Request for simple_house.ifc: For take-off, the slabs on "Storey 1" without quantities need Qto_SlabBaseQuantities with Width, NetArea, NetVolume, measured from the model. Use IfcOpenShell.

First a look at what the model holds.

```python
import ifcopenshell
import ifcopenshell.util.element
import ifcopenshell.util.unit

model = ifcopenshell.open("simple_house.ifc")
print(model.schema)
for unit_type in ("LENGTHUNIT", "AREAUNIT", "VOLUMEUNIT"):
    print(unit_type, ifcopenshell.util.unit.calculate_unit_scale(model, unit_type))
storey = next(s for s in model.by_type("IfcBuildingStorey") if s.Name == "Storey 1")
slabs = [e for e in ifcopenshell.util.element.get_decomposition(storey) if e.is_a("IfcSlab")]
for e in sorted(slabs, key=lambda e: e.id()):
    print(e.id(), e.is_a(), e.Name, list(ifcopenshell.util.element.get_psets(e, qtos_only=True)), sep=" | ")
```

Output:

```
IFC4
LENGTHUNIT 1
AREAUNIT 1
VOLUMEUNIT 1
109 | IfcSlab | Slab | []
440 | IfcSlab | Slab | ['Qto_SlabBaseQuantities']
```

```python
import ifcopenshell
import ifcopenshell.api.pset
import ifcopenshell.geom
import ifcopenshell.util.element
import ifcopenshell.util.shape
import ifcopenshell.util.unit

model = ifcopenshell.open("simple_house.ifc")
unit_scale = ifcopenshell.util.unit.calculate_unit_scale(model)
area_scale = ifcopenshell.util.unit.calculate_unit_scale(model, "AREAUNIT")
volume_scale = ifcopenshell.util.unit.calculate_unit_scale(model, "VOLUMEUNIT")
settings = ifcopenshell.geom.settings()

storey = next(s for s in model.by_type("IfcBuildingStorey") if s.Name == "Storey 1")
slabs = [e for e in ifcopenshell.util.element.get_decomposition(storey) if e.is_a("IfcSlab")]

for e in sorted(slabs, key=lambda e: e.id()):
    if ifcopenshell.util.element.get_psets(e, qtos_only=True, should_inherit=False):
        continue
    # Geometry comes back in metres, in the element's own axes.
    shape = ifcopenshell.geom.create_shape(settings, e)
    values = {
        "Width": ifcopenshell.util.shape.get_z(shape.geometry) / unit_scale,
        "NetArea": ifcopenshell.util.shape.get_footprint_area(shape.geometry) / area_scale,
        "NetVolume": ifcopenshell.util.shape.get_volume(shape.geometry) / volume_scale,
    }
    qto = ifcopenshell.api.pset.add_qto(model, product=e, name="Qto_SlabBaseQuantities")
    ifcopenshell.api.pset.edit_qto(model, qto=qto, properties=values)
    print(e.id(), {k: round(v, 3) for k, v in values.items()})

model.write("simple_house_v2.ifc")
```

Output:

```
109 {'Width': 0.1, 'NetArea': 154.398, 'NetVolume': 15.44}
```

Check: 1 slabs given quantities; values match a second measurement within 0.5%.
